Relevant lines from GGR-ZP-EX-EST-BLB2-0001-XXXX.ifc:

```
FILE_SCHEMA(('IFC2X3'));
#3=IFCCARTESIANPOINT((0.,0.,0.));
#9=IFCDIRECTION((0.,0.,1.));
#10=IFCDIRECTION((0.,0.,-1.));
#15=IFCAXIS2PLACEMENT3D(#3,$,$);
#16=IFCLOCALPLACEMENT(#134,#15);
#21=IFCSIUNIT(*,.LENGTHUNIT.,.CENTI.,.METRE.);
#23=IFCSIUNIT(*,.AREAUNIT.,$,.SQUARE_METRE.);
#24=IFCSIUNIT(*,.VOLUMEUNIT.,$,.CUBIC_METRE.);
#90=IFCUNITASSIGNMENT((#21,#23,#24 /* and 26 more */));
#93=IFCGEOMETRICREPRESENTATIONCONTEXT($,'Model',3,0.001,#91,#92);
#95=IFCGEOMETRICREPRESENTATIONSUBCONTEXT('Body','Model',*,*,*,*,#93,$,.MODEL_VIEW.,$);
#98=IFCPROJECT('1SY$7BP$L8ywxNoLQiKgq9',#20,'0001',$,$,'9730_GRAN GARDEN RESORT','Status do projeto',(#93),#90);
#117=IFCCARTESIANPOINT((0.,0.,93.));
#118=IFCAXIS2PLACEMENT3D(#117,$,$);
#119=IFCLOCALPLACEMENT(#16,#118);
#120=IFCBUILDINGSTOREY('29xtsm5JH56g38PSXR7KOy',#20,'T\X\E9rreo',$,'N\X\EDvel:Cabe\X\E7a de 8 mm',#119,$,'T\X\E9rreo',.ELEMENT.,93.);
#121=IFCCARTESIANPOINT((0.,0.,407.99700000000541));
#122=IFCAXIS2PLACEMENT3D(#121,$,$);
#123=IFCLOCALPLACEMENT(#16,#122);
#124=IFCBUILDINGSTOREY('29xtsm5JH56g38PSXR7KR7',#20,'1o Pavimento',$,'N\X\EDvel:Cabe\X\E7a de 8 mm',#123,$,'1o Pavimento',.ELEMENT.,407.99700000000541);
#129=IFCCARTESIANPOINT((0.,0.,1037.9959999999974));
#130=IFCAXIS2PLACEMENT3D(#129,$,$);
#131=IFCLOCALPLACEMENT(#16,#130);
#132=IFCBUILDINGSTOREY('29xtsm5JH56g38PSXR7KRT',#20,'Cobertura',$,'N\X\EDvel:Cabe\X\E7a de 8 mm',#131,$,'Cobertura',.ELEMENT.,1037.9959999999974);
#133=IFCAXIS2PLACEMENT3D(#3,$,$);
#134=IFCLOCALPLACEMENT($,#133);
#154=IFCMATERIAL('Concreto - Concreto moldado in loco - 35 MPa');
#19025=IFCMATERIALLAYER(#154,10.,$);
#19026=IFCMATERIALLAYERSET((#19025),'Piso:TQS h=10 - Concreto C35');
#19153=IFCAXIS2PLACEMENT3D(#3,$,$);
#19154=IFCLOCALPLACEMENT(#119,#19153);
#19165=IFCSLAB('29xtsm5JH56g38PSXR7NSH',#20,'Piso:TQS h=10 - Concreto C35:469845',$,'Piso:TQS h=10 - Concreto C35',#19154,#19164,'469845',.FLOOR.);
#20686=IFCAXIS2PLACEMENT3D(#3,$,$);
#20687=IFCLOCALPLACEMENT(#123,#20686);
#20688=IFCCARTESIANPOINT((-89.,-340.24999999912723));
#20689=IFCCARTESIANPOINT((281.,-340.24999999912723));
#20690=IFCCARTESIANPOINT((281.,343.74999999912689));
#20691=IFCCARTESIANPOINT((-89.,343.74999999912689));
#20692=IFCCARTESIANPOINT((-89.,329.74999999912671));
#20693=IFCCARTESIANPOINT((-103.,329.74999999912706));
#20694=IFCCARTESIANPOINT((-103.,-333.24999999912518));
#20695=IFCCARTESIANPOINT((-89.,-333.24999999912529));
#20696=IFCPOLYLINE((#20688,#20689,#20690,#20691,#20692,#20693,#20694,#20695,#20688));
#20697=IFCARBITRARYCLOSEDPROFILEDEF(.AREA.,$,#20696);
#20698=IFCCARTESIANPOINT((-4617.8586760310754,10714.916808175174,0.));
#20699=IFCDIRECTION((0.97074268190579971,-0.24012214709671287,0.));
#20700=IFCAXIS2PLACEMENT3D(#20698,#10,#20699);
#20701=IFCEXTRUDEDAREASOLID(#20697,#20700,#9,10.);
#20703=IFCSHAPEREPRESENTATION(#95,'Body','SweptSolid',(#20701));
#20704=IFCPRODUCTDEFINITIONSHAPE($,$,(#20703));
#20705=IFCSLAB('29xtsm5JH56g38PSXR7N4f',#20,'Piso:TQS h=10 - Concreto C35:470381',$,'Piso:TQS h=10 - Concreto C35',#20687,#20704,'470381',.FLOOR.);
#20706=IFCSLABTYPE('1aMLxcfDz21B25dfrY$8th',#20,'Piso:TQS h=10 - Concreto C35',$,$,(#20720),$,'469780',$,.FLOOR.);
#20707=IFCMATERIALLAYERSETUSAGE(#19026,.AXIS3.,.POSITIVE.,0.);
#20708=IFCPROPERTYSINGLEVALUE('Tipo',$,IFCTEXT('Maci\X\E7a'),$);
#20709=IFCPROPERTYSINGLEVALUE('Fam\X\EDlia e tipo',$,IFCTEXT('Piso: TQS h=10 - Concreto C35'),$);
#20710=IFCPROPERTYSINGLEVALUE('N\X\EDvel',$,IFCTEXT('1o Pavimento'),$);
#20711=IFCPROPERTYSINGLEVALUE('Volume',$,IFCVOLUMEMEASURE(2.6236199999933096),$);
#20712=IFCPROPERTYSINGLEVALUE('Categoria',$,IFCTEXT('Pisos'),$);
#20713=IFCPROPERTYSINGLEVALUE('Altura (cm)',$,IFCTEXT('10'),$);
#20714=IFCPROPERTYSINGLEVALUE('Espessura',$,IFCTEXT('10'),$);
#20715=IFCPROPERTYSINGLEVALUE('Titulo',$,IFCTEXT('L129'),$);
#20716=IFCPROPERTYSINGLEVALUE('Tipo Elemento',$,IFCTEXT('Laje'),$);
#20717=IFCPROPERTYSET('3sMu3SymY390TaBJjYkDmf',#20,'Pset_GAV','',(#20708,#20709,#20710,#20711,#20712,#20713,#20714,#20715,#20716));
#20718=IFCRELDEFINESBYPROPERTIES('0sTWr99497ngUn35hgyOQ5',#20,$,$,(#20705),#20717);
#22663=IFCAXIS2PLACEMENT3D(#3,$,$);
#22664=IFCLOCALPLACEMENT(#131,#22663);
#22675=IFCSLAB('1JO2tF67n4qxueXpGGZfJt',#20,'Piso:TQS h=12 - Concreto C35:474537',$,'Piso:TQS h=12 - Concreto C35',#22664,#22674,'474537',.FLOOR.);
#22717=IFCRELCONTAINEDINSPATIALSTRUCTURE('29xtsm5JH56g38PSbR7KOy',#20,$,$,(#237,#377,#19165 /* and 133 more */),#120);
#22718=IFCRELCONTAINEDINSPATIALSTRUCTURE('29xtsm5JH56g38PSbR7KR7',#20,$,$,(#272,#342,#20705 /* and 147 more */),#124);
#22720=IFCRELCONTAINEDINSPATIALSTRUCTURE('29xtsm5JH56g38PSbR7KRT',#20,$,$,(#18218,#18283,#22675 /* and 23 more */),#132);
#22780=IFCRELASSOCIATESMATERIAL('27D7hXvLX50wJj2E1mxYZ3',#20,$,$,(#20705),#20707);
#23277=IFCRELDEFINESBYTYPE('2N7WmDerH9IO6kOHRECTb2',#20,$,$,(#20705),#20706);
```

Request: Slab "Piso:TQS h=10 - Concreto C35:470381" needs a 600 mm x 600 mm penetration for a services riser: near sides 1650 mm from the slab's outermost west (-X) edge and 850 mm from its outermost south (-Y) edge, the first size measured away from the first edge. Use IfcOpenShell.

```python
import numpy as np
import ifcopenshell
import ifcopenshell.api.feature
import ifcopenshell.api.geometry
import ifcopenshell.api.pset
import ifcopenshell.api.root
import ifcopenshell.geom
import ifcopenshell.util.element
import ifcopenshell.util.placement
import ifcopenshell.util.representation
import ifcopenshell.util.shape
import ifcopenshell.util.unit

model = ifcopenshell.open("GGR-ZP-EX-EST-BLB2-0001-XXXX.ifc")
unit_scale = ifcopenshell.util.unit.calculate_unit_scale(model)
volume_scale = ifcopenshell.util.unit.calculate_unit_scale(model, "VOLUMEUNIT")
settings = ifcopenshell.geom.settings()


def volume(element):
    """Net volume in cubic metres, openings subtracted."""
    shape = ifcopenshell.geom.create_shape(settings, element)
    return ifcopenshell.util.shape.get_volume(shape.geometry)


slab = model.by_guid("29xtsm5JH56g38PSXR7N4f")
before = volume(slab)

# Extent in the slab's own axes, in metres. The edges named are its -X and -Y sides.
slab_shape = ifcopenshell.geom.create_shape(settings, slab)
vertices = ifcopenshell.util.shape.get_vertices(slab_shape.geometry)
x_min, y_min, bottom = vertices.min(axis=0)
top = vertices[:, 2].max()

opening = ifcopenshell.api.root.create_entity(model, ifc_class="IfcOpeningElement", name="Services riser opening")
context = ifcopenshell.util.representation.get_context(model, "Model", "Body", "MODEL_VIEW")
width, depth = 0.6, 0.6
outline = [(0.0, 0.0), (width, 0.0), (width, depth), (0.0, depth), (0.0, 0.0)]
# Overshoot both faces by 50 mm so the cut is clean.
shape = ifcopenshell.api.geometry.add_slab_representation(
    model, context=context, depth=top - bottom + 0.1, polyline=outline
)
ifcopenshell.api.geometry.assign_representation(model, product=opening, representation=shape)

matrix = ifcopenshell.util.placement.get_local_placement(slab.ObjectPlacement)
matrix[:, 3] = matrix @ np.append(np.array([x_min + 1.65, y_min + 0.85, bottom - 0.05]) / unit_scale, 1.0)
ifcopenshell.api.geometry.edit_object_placement(model, product=opening, matrix=matrix, is_si=False)
ifcopenshell.api.feature.add_feature(model, feature=opening, element=slab)

after = volume(slab)

# Update the slab's stored quantities.
pset = model.by_id(ifcopenshell.util.element.get_pset(slab, "Pset_GAV", should_inherit=False)["id"])
ifcopenshell.api.pset.edit_pset(model, pset=pset, properties={
    "Volume": model.create_entity("IfcVolumeMeasure", after / volume_scale),
})

print(f"slab volume {before:.3f} -> {after:.3f} m3")

model.write("GGR-ZP-EX-EST-BLB2-0001-XXXX_edited.ifc")
```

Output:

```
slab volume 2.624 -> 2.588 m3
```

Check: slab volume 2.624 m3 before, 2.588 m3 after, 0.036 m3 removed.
